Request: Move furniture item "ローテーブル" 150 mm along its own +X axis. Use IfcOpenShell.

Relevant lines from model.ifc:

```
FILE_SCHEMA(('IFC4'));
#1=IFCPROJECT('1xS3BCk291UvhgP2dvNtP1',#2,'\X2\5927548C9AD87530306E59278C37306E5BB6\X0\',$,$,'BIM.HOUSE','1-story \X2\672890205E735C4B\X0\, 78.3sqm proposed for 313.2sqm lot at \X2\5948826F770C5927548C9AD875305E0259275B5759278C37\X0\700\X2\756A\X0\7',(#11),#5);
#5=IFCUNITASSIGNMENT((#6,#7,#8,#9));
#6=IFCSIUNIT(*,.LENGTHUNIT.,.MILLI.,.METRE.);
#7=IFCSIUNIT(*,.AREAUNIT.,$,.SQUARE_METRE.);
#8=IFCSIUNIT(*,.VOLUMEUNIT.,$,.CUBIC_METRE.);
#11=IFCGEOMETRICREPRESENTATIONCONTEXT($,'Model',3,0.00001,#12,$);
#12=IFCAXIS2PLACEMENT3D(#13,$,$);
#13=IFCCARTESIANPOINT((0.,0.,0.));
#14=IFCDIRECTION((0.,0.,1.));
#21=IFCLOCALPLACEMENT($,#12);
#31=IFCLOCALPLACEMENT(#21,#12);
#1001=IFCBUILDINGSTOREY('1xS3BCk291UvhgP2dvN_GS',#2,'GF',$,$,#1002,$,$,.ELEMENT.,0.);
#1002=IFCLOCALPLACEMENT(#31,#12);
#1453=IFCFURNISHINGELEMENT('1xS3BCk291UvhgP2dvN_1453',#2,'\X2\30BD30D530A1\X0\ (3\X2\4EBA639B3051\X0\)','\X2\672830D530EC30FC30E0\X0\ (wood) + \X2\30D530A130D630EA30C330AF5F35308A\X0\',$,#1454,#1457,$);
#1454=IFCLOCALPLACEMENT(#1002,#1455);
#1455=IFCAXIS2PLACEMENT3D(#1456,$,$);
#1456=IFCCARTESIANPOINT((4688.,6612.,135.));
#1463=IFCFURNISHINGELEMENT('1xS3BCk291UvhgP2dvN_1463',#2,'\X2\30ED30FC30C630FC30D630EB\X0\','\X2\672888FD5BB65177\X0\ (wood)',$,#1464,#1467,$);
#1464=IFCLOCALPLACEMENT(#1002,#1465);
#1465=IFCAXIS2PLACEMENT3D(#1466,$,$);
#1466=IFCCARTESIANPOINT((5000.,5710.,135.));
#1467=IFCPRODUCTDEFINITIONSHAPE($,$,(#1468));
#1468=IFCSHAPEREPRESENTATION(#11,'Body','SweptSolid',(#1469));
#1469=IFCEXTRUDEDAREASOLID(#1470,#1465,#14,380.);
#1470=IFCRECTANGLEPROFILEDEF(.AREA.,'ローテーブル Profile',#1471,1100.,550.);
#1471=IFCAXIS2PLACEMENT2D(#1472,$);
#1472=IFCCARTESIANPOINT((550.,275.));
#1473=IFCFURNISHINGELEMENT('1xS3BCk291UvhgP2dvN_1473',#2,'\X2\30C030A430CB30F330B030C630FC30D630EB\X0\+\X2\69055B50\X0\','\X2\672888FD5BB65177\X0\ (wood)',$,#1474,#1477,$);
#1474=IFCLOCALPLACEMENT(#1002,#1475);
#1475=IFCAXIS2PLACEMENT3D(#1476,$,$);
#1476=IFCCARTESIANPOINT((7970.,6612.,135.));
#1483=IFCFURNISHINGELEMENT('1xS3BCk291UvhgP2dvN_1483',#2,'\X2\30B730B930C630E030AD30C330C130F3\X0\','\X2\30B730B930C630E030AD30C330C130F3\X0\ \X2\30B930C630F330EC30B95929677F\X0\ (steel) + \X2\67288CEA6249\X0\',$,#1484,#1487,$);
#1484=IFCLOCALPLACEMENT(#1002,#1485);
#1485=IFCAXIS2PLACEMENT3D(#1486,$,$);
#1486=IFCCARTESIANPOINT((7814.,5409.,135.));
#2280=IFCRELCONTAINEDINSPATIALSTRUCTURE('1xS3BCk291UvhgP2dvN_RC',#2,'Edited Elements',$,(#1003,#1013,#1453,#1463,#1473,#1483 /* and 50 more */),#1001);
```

```python
import ifcopenshell
import ifcopenshell.api.geometry
import ifcopenshell.util.placement

model = ifcopenshell.open("model.ifc")

item = model.by_guid("1xS3BCk291UvhgP2dvN_1463")
matrix = ifcopenshell.util.placement.get_local_placement(item.ObjectPlacement)
matrix[:3, 3] += matrix[:3, 0] * 150.0
ifcopenshell.api.geometry.edit_object_placement(model, product=item, matrix=matrix, is_si=False)

print(ifcopenshell.util.placement.get_local_placement(item.ObjectPlacement).round(3) + 0.0)

model.write("model_v2.ifc")
```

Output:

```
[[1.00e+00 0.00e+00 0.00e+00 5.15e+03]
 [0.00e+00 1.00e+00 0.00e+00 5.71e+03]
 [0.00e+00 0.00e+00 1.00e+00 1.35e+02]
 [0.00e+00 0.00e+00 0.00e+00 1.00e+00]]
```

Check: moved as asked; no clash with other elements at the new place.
